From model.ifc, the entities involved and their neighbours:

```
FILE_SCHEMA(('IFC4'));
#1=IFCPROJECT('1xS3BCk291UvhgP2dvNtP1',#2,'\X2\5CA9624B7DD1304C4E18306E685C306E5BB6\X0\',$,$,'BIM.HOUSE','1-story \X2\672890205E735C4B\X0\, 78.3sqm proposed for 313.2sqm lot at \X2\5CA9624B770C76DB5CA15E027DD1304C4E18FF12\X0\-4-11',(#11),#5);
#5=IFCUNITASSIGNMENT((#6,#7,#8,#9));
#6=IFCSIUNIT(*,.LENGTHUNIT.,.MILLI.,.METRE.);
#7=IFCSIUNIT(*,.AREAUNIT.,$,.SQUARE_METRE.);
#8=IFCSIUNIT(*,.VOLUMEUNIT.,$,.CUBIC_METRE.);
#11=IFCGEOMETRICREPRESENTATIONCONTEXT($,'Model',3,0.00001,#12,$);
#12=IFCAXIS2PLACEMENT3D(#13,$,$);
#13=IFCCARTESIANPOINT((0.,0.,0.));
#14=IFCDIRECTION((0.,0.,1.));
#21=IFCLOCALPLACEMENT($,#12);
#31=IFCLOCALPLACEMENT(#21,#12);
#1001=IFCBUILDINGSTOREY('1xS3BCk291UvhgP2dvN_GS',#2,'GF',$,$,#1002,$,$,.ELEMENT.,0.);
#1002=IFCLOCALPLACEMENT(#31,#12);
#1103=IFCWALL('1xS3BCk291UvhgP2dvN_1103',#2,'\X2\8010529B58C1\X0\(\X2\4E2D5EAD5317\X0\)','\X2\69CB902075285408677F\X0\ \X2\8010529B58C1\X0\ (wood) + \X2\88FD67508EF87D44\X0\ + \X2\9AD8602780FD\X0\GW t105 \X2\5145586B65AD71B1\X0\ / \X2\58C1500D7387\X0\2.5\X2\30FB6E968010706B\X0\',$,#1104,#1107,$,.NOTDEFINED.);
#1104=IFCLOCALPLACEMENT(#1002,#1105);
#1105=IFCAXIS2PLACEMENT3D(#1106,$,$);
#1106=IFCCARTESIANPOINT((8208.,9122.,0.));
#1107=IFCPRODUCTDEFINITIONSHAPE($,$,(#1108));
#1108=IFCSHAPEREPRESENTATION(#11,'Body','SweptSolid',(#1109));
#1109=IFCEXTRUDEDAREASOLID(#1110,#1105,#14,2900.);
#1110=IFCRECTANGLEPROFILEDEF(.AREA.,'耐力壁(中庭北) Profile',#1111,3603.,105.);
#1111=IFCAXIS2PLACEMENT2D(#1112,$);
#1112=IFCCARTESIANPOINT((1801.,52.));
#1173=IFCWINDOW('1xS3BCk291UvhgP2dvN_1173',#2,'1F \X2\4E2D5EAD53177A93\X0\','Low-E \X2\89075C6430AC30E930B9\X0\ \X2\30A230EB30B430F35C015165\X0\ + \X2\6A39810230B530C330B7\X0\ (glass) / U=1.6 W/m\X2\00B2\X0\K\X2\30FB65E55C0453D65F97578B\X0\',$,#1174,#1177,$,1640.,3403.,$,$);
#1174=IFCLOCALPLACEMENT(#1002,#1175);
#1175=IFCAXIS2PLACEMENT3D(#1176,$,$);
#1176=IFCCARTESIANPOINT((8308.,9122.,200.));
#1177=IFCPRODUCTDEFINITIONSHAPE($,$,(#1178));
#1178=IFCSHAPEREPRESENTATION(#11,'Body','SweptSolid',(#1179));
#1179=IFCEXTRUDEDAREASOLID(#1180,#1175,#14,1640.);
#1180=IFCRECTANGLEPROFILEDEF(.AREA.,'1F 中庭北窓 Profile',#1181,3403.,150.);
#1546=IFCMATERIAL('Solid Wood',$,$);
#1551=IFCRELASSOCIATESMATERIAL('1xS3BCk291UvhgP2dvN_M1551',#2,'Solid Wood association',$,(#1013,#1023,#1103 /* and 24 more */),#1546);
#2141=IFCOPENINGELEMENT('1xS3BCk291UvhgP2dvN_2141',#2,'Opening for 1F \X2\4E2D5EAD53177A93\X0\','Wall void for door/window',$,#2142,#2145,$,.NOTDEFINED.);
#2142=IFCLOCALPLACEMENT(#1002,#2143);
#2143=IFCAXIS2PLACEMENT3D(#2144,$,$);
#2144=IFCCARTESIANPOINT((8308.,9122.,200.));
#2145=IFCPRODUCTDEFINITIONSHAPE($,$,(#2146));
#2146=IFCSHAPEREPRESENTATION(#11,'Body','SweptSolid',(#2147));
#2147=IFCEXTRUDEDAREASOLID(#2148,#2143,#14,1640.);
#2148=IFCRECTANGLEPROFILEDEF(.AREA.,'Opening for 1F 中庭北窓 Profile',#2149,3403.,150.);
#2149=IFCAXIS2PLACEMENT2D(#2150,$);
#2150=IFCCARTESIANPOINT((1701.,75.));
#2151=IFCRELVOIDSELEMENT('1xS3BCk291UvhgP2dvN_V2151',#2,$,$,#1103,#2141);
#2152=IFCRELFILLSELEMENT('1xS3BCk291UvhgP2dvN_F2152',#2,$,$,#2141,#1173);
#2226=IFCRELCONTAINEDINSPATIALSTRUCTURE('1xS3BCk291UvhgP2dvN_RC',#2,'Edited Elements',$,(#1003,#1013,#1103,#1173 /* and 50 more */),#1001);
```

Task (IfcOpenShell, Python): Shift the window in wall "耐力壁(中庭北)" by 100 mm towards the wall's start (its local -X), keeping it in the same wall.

```python
import ifcopenshell
import ifcopenshell.api.geometry
import ifcopenshell.util.placement

model = ifcopenshell.open("model.ifc")

window = model.by_guid("1xS3BCk291UvhgP2dvN_1173")
opening = window.FillsVoids[0].RelatingOpeningElement
wall = opening.VoidsElements[0].RelatingBuildingElement

wall_matrix = ifcopenshell.util.placement.get_local_placement(wall.ObjectPlacement)
shift = wall_matrix[:3, 0] * -100.0
before = ifcopenshell.util.placement.get_local_placement(window.ObjectPlacement)[:3, 3].copy()

# The window is not placed relative to its opening, so move both.
for product in (opening, window):
    matrix = ifcopenshell.util.placement.get_local_placement(product.ObjectPlacement)
    matrix[:3, 3] += shift
    ifcopenshell.api.geometry.edit_object_placement(model, product=product, matrix=matrix, is_si=False)

after = ifcopenshell.util.placement.get_local_placement(window.ObjectPlacement)[:3, 3]
print("window moved by", (after - before).round(3) + 0.0)

model.write("model_updated.ifc")
```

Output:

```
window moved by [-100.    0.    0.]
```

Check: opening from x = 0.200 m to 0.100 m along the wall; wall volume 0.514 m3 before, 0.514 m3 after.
